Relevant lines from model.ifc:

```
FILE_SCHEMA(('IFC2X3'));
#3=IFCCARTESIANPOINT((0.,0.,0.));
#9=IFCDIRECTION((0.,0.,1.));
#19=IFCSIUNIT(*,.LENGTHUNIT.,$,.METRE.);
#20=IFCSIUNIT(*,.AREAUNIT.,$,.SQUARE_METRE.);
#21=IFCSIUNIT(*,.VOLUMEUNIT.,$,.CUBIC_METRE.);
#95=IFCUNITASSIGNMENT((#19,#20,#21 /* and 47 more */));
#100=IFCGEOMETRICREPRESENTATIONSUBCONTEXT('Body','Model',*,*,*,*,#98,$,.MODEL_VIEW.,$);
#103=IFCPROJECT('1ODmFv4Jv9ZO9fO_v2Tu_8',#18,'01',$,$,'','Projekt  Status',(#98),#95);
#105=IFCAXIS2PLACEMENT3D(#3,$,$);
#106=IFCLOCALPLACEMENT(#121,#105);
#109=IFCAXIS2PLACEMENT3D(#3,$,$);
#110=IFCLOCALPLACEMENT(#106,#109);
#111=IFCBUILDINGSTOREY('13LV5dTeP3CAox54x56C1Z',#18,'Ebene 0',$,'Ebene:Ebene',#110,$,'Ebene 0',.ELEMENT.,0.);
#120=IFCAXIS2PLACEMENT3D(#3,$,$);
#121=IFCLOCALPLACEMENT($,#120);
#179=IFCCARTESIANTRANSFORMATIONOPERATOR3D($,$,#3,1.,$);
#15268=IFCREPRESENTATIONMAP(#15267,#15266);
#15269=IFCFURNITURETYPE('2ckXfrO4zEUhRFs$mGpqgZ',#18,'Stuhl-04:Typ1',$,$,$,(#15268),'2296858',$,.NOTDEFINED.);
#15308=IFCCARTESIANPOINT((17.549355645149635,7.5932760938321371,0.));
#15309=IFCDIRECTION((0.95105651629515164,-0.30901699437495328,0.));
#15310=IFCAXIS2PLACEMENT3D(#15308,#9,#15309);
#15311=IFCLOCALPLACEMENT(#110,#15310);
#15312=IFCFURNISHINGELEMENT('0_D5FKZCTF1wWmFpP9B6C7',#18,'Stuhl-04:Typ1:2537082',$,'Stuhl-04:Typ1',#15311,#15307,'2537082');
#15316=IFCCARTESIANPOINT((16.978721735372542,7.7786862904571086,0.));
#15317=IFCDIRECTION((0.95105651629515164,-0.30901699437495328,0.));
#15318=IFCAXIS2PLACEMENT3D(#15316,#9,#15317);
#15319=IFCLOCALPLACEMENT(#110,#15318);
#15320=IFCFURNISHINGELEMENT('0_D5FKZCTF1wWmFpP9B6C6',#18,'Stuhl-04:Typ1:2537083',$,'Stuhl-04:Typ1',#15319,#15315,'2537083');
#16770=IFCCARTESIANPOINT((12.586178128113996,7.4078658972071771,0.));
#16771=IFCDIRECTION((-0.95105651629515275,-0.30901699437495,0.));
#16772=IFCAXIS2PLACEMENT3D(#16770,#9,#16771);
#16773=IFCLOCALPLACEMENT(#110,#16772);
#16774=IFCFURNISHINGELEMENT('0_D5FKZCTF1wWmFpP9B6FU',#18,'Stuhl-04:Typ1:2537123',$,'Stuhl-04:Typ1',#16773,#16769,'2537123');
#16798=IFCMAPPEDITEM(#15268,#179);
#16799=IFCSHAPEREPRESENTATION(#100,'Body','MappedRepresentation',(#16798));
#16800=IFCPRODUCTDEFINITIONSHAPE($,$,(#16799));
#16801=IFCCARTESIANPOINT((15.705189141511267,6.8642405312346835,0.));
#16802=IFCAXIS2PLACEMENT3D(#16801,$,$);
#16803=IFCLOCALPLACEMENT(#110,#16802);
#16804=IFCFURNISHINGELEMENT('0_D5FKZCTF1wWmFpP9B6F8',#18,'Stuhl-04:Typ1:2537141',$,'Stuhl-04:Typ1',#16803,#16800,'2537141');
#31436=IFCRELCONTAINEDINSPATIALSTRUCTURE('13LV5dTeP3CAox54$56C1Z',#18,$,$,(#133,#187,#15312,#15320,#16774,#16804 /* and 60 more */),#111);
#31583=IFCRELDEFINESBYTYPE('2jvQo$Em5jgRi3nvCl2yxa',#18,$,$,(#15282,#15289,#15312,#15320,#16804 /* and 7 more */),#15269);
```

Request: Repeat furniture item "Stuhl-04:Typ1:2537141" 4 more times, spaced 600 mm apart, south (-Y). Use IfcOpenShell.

```python
import numpy as np
import ifcopenshell
import ifcopenshell.api.geometry
import ifcopenshell.api.root
import ifcopenshell.util.element
import ifcopenshell.util.placement
import ifcopenshell.util.unit

model = ifcopenshell.open("model.ifc")
unit_scale = ifcopenshell.util.unit.calculate_unit_scale(model)

source = model.by_guid("0_D5FKZCTF1wWmFpP9B6F8")
base = ifcopenshell.util.placement.get_local_placement(source.ObjectPlacement)
step = np.array([0.0, -1.0, 0.0]) * 0.6 / unit_scale

for i in range(1, 5):
    copy = ifcopenshell.api.root.copy_class(model, product=source)
    copy.Representation = ifcopenshell.util.element.copy_deep(
        model, source.Representation, exclude=["IfcGeometricRepresentationContext", "IfcRepresentationMap"]
    )
    copy.Name = "Stuhl-04:Typ1"
    copy.Tag = None
    matrix = base.copy()
    matrix[:3, 3] += i * step
    print("added at", matrix[:3, 3].round(3) + 0.0)
    ifcopenshell.api.geometry.edit_object_placement(model, product=copy, matrix=matrix, is_si=False)

model.write("model_v2.ifc")
```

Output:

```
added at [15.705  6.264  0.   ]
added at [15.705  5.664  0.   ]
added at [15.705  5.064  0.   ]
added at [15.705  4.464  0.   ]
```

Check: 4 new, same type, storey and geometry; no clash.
